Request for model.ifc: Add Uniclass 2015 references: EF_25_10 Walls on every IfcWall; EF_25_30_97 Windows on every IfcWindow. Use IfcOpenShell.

First a look at what the model holds.

```python
import ifcopenshell

model = ifcopenshell.open("model.ifc")
print(model.schema)
print("classifications:", [c.Name for c in model.by_type("IfcClassification")])
for ifc_class in ("IfcDoor", "IfcRoof", "IfcStair", "IfcWall", "IfcWindow"):
    print(ifc_class, len(model.by_type(ifc_class)))
```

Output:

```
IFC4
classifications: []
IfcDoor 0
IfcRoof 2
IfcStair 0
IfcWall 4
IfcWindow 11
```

```python
import ifcopenshell
import ifcopenshell.api.classification

model = ifcopenshell.open("model.ifc")

system = ifcopenshell.api.classification.add_classification(model, classification="Uniclass 2015")

codes = {
    "IfcWall": ("EF_25_10", "Walls"),
    "IfcWindow": ("EF_25_30_97", "Windows"),
}
for ifc_class, (code, name) in codes.items():
    products = model.by_type(ifc_class)
    ifcopenshell.api.classification.add_reference(
        model, products=products, classification=system, identification=code, name=name
    )
    print(code, len(products))

model.write("model_v2.ifc")
```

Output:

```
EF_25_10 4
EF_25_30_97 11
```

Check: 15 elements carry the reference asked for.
